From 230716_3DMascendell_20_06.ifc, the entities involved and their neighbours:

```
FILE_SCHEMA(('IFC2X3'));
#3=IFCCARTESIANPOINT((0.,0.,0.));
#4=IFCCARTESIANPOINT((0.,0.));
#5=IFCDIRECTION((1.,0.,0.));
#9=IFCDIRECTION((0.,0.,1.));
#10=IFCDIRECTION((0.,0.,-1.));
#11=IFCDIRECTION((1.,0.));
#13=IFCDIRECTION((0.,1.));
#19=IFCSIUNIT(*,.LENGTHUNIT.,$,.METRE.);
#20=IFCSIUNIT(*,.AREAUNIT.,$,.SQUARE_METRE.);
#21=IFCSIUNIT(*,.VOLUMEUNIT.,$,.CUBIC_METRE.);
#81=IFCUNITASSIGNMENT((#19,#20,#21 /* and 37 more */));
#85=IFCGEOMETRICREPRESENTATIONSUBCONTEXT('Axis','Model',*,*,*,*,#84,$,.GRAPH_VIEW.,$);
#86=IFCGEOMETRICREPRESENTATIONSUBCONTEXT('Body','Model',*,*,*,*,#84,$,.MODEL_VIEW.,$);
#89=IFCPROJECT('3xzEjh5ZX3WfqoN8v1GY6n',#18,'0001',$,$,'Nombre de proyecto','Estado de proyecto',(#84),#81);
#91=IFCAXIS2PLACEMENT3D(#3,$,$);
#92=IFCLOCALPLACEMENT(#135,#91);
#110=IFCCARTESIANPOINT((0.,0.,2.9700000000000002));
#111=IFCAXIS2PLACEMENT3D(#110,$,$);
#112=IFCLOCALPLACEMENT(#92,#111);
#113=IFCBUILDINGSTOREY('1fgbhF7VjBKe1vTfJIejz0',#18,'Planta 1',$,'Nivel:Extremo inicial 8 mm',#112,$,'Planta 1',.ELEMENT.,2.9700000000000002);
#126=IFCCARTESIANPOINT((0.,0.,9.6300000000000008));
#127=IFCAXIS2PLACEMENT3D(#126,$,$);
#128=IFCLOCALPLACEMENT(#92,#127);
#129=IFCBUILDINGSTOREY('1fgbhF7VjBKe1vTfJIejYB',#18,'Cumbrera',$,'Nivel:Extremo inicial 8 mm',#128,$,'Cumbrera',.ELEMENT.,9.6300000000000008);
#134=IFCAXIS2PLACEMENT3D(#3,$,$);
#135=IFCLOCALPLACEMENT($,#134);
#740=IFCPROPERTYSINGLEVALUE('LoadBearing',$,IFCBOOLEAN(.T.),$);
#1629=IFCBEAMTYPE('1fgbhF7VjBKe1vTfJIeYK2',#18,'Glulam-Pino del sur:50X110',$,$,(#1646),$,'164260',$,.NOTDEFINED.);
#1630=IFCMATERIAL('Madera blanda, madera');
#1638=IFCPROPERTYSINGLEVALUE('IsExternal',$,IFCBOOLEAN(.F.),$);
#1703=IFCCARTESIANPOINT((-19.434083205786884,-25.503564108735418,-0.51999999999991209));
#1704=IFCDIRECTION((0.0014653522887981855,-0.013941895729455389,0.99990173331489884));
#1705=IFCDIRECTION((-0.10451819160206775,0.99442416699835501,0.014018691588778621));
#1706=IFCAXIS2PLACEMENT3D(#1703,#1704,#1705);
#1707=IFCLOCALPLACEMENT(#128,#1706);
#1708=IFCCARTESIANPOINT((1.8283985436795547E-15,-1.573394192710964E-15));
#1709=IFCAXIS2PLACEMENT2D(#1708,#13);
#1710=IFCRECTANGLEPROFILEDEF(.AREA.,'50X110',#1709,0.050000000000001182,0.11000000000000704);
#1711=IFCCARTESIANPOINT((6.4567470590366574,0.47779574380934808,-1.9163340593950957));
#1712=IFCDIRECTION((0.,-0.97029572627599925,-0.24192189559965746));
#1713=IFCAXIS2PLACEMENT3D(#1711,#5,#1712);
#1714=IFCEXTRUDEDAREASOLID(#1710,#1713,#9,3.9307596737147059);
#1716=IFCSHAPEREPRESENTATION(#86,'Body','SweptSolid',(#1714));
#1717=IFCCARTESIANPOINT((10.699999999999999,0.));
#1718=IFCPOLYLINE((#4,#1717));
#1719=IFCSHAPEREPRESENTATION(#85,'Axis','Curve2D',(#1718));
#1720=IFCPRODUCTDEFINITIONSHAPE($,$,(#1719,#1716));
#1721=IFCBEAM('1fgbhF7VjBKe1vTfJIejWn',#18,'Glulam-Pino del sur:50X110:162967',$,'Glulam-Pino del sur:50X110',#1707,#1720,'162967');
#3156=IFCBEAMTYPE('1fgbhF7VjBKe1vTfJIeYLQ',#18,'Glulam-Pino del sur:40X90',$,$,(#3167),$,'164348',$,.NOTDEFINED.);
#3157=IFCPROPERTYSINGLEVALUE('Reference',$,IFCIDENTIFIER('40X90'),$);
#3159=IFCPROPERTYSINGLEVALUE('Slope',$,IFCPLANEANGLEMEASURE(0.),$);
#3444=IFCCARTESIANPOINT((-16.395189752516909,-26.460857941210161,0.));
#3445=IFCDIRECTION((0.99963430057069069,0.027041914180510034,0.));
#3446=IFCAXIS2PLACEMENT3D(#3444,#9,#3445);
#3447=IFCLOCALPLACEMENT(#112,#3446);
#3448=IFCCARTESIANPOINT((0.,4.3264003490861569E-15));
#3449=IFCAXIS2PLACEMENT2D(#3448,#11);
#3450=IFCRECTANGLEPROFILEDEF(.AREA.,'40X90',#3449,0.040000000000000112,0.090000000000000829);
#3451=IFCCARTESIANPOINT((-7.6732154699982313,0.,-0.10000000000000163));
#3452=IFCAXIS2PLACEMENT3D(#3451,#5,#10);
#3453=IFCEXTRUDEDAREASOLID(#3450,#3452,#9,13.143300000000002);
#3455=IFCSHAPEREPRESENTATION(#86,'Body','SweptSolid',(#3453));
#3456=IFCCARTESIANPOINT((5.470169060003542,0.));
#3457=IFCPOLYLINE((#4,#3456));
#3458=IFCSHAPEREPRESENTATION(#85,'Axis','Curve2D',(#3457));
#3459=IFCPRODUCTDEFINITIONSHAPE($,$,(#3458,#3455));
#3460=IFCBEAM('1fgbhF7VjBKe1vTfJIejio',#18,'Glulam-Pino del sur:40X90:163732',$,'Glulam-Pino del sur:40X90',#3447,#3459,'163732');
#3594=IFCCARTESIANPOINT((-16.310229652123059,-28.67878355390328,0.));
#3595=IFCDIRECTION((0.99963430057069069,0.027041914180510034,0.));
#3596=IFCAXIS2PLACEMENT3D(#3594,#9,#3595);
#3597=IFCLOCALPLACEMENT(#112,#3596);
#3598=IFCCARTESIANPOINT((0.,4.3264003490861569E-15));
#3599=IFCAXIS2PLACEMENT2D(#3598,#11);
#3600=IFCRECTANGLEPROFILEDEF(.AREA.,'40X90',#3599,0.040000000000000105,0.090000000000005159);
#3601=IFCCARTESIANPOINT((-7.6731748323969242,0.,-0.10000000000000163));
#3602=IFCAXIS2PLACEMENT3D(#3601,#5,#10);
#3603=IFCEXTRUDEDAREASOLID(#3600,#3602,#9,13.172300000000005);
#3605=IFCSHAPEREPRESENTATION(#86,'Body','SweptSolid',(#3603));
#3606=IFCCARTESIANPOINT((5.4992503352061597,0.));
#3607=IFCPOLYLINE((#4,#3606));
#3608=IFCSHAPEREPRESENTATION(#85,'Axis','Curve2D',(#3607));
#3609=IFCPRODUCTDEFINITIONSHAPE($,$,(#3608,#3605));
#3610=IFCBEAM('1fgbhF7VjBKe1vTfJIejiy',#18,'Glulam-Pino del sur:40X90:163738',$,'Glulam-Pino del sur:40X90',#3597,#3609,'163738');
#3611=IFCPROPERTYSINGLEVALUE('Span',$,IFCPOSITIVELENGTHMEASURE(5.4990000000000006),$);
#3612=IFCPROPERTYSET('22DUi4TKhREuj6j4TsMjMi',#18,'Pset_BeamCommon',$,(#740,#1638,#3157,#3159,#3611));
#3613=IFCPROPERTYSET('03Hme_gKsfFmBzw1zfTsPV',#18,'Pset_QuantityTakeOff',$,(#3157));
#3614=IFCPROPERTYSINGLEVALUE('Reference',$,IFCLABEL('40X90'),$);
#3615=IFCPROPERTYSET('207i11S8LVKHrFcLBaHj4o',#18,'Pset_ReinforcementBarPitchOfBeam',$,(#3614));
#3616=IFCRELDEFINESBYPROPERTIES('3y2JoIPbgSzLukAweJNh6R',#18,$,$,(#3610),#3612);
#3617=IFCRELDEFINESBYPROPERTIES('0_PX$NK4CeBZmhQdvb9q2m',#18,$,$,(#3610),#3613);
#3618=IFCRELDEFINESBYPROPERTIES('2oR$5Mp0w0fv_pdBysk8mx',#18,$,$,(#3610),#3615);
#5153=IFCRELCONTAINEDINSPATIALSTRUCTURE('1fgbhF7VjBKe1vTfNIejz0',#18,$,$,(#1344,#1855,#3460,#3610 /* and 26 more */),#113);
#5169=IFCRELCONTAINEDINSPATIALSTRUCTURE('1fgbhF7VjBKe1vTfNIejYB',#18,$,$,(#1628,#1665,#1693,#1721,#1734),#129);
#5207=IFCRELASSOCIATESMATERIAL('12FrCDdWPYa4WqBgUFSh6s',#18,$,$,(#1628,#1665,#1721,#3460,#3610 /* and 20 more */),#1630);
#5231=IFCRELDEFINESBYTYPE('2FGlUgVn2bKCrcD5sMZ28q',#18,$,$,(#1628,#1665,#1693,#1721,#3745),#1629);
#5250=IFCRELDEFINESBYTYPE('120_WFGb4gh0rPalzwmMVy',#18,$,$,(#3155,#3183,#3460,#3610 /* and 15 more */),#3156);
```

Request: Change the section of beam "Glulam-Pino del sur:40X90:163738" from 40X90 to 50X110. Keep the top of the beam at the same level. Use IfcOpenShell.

```python
import ifcopenshell
import ifcopenshell.api.pset
import ifcopenshell.api.type
import ifcopenshell.util.element
import ifcopenshell.util.representation

model = ifcopenshell.open("230716_3DMascendell_20_06.ifc")

member = model.by_guid("1fgbhF7VjBKe1vTfJIejiy")
source = next(p for p in model.by_type("IfcRectangleProfileDef") if p.ProfileName == "50X110")

body = ifcopenshell.util.representation.get_representation(member, "Model", "Body")
solid = body.Items[0]
old_profile = solid.SweptArea

# Copy the section's sizes but keep this member's own profile position.
profile = ifcopenshell.util.element.copy(model, source)
# Profiles are centred, so shift by half the change in depth to hold the top.
shift = (old_profile.XDim - profile.XDim) / 2
x, y = old_profile.Position.Location.Coordinates
up = (-1.0, 0.0)  # upwards, in the solid's own plane
location = model.createIfcCartesianPoint((x + up[0] * shift, y + up[1] * shift))
profile.Position = model.createIfcAxis2Placement2D(location, old_profile.Position.RefDirection)
solid.SweptArea = profile
if not model.get_total_inverses(old_profile):
    ifcopenshell.util.element.remove_deep2(model, old_profile)

new_type = model.by_id(1629)
ifcopenshell.api.type.assign_type(
    model, related_objects=[member], relating_type=new_type, should_map_representations=False
)
member.Name = member.Name.replace("40X90", "50X110")
member.ObjectType = "Glulam-Pino del sur:50X110"
pset = model.by_id(ifcopenshell.util.element.get_pset(member, "Pset_BeamCommon", should_inherit=False)["id"])
ifcopenshell.api.pset.edit_pset(model, pset=pset, properties={"Reference": "50X110"})
pset = model.by_id(ifcopenshell.util.element.get_pset(member, "Pset_QuantityTakeOff", should_inherit=False)["id"])
ifcopenshell.api.pset.edit_pset(model, pset=pset, properties={"Reference": "50X110"})
pset = model.by_id(ifcopenshell.util.element.get_pset(member, "Pset_ReinforcementBarPitchOfBeam", should_inherit=False)["id"])
ifcopenshell.api.pset.edit_pset(model, pset=pset, properties={"Reference": "50X110"})

print(solid.SweptArea)

model.write("230716_3DMascendell_20_06_edited.ifc")
```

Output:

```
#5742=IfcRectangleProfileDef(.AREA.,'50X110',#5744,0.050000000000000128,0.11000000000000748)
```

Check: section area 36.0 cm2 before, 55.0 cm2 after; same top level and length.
